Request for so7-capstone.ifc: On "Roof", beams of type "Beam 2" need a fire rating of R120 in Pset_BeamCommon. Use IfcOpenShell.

First a look at what the model holds.

```python
import ifcopenshell
import ifcopenshell.util.element

model = ifcopenshell.open("so7-capstone.ifc")
print(model.schema)
storey = next(s for s in model.by_type("IfcBuildingStorey") if s.Name == "Roof")
beams = [e for e in ifcopenshell.util.element.get_decomposition(storey) if e.is_a("IfcBeam")]
seen = {}
for e in beams:
    element_type = ifcopenshell.util.element.get_type(e)
    key = (element_type.Name if element_type != e and element_type else None, ifcopenshell.util.element.get_pset(e, "Pset_BeamCommon", "FireRating"))
    seen[key] = seen.get(key, 0) + 1
for (name, value), count in sorted(seen.items(), key=str):
    print(count, "x", name, "|", value)
```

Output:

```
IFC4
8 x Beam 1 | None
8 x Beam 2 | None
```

```python
import ifcopenshell
import ifcopenshell.api.pset
import ifcopenshell.util.element

model = ifcopenshell.open("so7-capstone.ifc")

storey = next(s for s in model.by_type("IfcBuildingStorey") if s.Name == "Roof")
beams = [e for e in ifcopenshell.util.element.get_decomposition(storey) if e.is_a("IfcBeam")]

count = 0
for e in beams:
    element_type = ifcopenshell.util.element.get_type(e)
    if element_type in (None, e) or element_type.Name != "Beam 2":
        continue
    # add_pset returns the element's existing set when there is one.
    pset = ifcopenshell.api.pset.add_pset(model, product=e, name="Pset_BeamCommon")
    ifcopenshell.api.pset.edit_pset(model, pset=pset, properties={"FireRating": "R120"})
    count += 1

print(count, "beams updated")

model.write("so7-capstone_updated.ifc")
```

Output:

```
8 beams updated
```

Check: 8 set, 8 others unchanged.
